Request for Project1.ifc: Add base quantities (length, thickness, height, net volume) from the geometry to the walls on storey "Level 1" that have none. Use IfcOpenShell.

First a look at what the model holds.

```python
import ifcopenshell
import ifcopenshell.util.element
import ifcopenshell.util.unit

model = ifcopenshell.open("Project1.ifc")
print(model.schema)
for unit_type in ("LENGTHUNIT", "AREAUNIT", "VOLUMEUNIT"):
    print(unit_type, ifcopenshell.util.unit.calculate_unit_scale(model, unit_type))
storey = next(s for s in model.by_type("IfcBuildingStorey") if s.Name == "Level 1")
walls = [e for e in ifcopenshell.util.element.get_decomposition(storey) if e.is_a("IfcWall")]
for e in sorted(walls, key=lambda e: e.id()):
    print(e.id(), e.is_a(), e.Name, list(ifcopenshell.util.element.get_psets(e, qtos_only=True)), sep=" | ")
```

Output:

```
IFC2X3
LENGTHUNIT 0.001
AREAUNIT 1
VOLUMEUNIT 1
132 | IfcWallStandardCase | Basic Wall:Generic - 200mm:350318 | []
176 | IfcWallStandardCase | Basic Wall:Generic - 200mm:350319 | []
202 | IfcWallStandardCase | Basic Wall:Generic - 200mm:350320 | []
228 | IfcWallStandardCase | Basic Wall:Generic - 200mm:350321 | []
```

```python
import ifcopenshell
import ifcopenshell.api.pset
import ifcopenshell.geom
import ifcopenshell.util.element
import ifcopenshell.util.shape
import ifcopenshell.util.unit

model = ifcopenshell.open("Project1.ifc")
unit_scale = ifcopenshell.util.unit.calculate_unit_scale(model)
volume_scale = ifcopenshell.util.unit.calculate_unit_scale(model, "VOLUMEUNIT")
settings = ifcopenshell.geom.settings()

storey = next(s for s in model.by_type("IfcBuildingStorey") if s.Name == "Level 1")
walls = [e for e in ifcopenshell.util.element.get_decomposition(storey) if e.is_a("IfcWall")]

for e in sorted(walls, key=lambda e: e.id()):
    if ifcopenshell.util.element.get_psets(e, qtos_only=True, should_inherit=False):
        continue
    # Geometry comes back in metres, in the element's own axes.
    shape = ifcopenshell.geom.create_shape(settings, e)
    values = {
        "Length": ifcopenshell.util.shape.get_x(shape.geometry) / unit_scale,
        "Width": ifcopenshell.util.shape.get_y(shape.geometry) / unit_scale,
        "Height": ifcopenshell.util.shape.get_z(shape.geometry) / unit_scale,
        "NetVolume": ifcopenshell.util.shape.get_volume(shape.geometry) / volume_scale,
    }
    qto = ifcopenshell.api.pset.add_qto(model, product=e, name="BaseQuantities")
    ifcopenshell.api.pset.edit_qto(model, qto=qto, properties=values)
    print(e.id(), {k: round(v, 3) for k, v in values.items()})

model.write("Project1_v2.ifc")
```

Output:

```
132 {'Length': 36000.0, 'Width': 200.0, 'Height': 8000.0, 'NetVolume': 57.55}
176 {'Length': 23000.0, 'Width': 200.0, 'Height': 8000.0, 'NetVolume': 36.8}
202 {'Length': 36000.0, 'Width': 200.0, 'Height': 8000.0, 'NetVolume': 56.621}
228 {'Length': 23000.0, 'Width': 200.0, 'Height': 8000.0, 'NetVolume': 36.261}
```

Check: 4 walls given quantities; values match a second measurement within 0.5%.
